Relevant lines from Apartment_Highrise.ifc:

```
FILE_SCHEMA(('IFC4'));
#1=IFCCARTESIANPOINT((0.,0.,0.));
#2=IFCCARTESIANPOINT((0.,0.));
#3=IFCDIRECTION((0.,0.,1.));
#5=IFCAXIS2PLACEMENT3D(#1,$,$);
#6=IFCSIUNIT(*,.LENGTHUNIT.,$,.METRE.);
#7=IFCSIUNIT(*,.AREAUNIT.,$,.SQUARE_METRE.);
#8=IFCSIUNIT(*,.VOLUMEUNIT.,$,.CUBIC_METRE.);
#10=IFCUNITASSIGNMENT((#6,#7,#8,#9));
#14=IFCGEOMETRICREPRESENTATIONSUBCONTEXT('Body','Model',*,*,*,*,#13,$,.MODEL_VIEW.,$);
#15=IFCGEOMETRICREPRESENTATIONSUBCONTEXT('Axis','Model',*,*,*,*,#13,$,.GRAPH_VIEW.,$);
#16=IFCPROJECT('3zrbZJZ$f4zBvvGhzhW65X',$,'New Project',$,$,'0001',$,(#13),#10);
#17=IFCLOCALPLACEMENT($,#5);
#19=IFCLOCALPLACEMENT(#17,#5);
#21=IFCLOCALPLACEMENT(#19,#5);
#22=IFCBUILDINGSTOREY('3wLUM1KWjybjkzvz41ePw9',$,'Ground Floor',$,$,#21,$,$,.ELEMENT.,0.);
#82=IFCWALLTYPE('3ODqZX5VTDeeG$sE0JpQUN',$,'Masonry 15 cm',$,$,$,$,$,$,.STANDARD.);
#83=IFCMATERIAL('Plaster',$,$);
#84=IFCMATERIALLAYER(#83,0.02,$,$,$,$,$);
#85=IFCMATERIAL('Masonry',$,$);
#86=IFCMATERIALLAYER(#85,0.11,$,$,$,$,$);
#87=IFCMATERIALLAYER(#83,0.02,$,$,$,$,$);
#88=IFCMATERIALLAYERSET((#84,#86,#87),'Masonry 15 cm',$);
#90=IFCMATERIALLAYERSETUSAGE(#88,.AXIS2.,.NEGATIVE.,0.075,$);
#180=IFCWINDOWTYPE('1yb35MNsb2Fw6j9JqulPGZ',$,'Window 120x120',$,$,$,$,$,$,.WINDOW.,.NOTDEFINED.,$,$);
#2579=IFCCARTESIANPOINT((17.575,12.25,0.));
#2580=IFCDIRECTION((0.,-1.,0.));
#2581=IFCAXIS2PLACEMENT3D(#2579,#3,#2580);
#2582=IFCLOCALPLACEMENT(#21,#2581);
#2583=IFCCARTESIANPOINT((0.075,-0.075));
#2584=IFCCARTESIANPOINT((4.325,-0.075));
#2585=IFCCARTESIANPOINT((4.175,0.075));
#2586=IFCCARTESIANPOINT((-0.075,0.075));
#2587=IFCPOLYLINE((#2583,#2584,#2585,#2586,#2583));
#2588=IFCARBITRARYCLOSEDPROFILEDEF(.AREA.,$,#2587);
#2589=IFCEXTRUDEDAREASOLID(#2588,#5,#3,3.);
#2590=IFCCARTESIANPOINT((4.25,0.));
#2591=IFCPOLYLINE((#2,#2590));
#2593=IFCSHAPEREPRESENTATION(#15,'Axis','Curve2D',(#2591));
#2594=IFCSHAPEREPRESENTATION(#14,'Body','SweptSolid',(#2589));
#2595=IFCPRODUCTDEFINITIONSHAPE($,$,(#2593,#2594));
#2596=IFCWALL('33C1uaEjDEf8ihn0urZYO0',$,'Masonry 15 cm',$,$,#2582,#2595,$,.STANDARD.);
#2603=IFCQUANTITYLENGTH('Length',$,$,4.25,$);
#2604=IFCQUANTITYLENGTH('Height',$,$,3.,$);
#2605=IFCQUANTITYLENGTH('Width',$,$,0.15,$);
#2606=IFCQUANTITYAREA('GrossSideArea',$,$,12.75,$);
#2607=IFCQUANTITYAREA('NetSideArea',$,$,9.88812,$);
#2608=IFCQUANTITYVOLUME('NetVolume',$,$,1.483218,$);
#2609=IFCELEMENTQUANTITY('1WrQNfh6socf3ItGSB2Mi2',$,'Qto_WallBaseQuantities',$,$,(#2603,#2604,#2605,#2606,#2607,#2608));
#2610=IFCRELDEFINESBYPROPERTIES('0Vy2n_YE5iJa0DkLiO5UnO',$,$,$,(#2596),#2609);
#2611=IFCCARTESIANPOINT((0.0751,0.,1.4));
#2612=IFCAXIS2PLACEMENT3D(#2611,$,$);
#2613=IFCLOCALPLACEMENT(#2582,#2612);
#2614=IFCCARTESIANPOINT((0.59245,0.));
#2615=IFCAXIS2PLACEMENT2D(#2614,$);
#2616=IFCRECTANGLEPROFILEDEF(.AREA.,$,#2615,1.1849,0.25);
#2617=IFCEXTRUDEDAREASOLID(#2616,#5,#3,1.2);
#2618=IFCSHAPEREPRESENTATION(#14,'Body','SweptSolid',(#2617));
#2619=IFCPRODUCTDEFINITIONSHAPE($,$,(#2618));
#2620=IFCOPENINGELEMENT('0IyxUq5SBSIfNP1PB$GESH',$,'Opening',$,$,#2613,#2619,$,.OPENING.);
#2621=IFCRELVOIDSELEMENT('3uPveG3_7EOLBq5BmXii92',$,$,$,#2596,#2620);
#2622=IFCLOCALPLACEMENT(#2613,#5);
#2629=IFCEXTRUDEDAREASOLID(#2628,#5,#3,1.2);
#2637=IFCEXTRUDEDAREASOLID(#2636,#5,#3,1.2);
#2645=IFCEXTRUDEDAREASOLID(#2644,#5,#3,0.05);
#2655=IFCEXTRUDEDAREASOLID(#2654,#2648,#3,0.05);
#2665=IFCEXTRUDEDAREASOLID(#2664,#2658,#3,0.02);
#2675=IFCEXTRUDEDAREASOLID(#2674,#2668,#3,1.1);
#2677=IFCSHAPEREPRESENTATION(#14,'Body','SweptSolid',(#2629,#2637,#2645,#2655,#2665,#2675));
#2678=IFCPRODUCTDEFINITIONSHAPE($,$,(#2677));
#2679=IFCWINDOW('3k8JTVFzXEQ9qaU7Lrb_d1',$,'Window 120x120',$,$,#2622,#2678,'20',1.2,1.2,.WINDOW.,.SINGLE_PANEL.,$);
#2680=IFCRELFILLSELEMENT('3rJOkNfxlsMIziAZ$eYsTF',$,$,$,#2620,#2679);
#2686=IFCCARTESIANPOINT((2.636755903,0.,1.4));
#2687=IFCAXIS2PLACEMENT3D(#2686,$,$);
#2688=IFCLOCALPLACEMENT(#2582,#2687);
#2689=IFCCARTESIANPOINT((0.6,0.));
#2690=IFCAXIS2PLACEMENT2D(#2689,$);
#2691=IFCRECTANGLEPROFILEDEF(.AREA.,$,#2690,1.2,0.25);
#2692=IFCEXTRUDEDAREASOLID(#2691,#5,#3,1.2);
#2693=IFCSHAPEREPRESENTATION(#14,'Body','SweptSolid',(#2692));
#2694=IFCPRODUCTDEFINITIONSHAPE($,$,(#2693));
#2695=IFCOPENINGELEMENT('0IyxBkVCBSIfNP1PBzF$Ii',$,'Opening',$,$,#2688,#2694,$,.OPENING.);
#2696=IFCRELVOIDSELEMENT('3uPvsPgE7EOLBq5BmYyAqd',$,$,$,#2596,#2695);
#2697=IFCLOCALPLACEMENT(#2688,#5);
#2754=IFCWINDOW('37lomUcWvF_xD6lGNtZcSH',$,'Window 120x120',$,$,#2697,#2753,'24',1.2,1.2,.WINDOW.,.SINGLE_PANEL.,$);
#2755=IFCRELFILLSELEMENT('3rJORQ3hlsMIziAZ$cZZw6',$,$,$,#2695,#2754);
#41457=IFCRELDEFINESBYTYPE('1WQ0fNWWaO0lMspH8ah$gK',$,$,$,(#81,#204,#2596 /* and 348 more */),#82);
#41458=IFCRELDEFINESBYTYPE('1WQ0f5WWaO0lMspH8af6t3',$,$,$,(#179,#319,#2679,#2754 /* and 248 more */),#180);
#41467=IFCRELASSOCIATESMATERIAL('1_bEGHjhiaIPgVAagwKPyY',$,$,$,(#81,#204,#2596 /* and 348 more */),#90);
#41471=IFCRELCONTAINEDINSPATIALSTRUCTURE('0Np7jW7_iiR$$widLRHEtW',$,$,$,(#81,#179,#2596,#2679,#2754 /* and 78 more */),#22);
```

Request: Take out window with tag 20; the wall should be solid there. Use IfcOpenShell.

```python
import ifcopenshell
import ifcopenshell.api.feature
import ifcopenshell.api.pset
import ifcopenshell.api.root
import ifcopenshell.geom
import ifcopenshell.util.element
import ifcopenshell.util.shape
import ifcopenshell.util.unit

model = ifcopenshell.open("Apartment_Highrise.ifc")
area_scale = ifcopenshell.util.unit.calculate_unit_scale(model, "AREAUNIT")
volume_scale = ifcopenshell.util.unit.calculate_unit_scale(model, "VOLUMEUNIT")
settings = ifcopenshell.geom.settings()


def volume(element):
    """Net volume in cubic metres, openings subtracted."""
    shape = ifcopenshell.geom.create_shape(settings, element)
    return ifcopenshell.util.shape.get_volume(shape.geometry)


window = model.by_id(2679)
opening = window.FillsVoids[0].RelatingOpeningElement
wall = opening.VoidsElements[0].RelatingBuildingElement
before = volume(wall)

ifcopenshell.api.root.remove_product(model, product=window)
ifcopenshell.api.feature.remove_feature(model, feature=opening)

after = volume(wall)
thickness = 0.15  # wall thickness in metres

# Update the wall's stored quantities.
qto = model.by_id(ifcopenshell.util.element.get_pset(wall, "Qto_WallBaseQuantities", should_inherit=False)["id"])
ifcopenshell.api.pset.edit_qto(model, qto=qto, properties={
    "NetSideArea": after / thickness / area_scale,
    "NetVolume": after / volume_scale,
})

print(f"wall volume {before:.3f} -> {after:.3f} m3")

model.write("Apartment_Highrise_updated.ifc")
```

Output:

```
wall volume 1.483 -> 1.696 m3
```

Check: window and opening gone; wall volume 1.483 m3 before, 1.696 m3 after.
